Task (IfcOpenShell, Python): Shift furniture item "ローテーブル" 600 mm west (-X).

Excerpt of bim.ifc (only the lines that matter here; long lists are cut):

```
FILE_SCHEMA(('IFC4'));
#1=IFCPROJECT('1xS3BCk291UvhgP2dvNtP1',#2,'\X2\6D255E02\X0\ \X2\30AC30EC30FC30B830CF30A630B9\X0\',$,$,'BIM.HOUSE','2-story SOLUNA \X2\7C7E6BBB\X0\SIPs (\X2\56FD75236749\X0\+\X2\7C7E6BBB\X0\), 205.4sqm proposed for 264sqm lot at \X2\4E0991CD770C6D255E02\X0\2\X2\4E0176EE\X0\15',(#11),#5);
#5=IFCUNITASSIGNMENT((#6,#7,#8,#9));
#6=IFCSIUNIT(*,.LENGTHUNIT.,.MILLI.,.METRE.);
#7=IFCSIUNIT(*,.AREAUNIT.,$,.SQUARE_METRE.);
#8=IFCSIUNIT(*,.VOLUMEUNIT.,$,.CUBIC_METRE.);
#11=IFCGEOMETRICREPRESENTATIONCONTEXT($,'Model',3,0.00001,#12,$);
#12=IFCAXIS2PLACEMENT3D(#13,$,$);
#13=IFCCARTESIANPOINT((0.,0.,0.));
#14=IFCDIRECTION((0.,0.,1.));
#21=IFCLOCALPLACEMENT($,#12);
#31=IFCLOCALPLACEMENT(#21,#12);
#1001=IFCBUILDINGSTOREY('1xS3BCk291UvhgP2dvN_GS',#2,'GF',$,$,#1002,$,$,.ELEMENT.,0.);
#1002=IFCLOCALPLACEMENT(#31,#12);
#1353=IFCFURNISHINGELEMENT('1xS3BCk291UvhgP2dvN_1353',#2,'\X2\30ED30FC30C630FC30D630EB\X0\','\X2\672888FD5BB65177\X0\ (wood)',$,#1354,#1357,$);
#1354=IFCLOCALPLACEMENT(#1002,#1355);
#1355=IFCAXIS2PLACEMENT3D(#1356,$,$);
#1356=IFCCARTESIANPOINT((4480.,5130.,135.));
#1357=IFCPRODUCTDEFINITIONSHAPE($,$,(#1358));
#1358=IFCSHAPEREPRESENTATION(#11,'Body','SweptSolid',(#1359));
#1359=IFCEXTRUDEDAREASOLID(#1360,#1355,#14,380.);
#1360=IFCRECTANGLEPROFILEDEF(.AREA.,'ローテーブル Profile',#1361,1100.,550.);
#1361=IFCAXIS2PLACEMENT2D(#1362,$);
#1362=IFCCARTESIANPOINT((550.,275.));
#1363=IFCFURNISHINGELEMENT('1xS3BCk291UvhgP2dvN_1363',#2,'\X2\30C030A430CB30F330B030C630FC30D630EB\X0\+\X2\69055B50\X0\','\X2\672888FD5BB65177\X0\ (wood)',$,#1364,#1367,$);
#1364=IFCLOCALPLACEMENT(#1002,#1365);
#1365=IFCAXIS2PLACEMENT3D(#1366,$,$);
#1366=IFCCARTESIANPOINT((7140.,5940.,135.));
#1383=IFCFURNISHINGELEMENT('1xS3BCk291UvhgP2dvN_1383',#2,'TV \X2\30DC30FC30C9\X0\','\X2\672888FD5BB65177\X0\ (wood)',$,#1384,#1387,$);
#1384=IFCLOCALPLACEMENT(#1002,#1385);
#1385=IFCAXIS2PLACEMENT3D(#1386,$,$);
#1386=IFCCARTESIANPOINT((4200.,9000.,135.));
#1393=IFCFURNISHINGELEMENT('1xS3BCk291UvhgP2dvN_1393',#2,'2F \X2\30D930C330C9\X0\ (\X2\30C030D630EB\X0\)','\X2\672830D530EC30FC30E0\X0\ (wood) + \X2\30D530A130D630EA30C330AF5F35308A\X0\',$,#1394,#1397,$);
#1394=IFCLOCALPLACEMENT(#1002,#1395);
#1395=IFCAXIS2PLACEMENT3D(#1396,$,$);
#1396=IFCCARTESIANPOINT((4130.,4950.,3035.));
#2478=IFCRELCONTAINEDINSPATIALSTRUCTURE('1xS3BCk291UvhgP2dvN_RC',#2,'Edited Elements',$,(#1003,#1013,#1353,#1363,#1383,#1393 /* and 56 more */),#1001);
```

```python
import ifcopenshell
import ifcopenshell.api.geometry
import ifcopenshell.util.placement
import ifcopenshell.util.unit

model = ifcopenshell.open("bim.ifc")
unit_scale = ifcopenshell.util.unit.calculate_unit_scale(model)

item = model.by_guid("1xS3BCk291UvhgP2dvN_1353")
matrix = ifcopenshell.util.placement.get_local_placement(item.ObjectPlacement)
matrix[0, 3] -= 0.6 / unit_scale
ifcopenshell.api.geometry.edit_object_placement(model, product=item, matrix=matrix, is_si=False)

print(ifcopenshell.util.placement.get_local_placement(item.ObjectPlacement).round(3) + 0.0)

model.write("bim_edited.ifc")
```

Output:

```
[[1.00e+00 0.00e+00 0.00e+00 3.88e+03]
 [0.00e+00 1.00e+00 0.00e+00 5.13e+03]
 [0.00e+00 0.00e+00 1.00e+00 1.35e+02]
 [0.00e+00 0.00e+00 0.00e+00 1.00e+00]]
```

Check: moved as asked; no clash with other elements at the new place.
